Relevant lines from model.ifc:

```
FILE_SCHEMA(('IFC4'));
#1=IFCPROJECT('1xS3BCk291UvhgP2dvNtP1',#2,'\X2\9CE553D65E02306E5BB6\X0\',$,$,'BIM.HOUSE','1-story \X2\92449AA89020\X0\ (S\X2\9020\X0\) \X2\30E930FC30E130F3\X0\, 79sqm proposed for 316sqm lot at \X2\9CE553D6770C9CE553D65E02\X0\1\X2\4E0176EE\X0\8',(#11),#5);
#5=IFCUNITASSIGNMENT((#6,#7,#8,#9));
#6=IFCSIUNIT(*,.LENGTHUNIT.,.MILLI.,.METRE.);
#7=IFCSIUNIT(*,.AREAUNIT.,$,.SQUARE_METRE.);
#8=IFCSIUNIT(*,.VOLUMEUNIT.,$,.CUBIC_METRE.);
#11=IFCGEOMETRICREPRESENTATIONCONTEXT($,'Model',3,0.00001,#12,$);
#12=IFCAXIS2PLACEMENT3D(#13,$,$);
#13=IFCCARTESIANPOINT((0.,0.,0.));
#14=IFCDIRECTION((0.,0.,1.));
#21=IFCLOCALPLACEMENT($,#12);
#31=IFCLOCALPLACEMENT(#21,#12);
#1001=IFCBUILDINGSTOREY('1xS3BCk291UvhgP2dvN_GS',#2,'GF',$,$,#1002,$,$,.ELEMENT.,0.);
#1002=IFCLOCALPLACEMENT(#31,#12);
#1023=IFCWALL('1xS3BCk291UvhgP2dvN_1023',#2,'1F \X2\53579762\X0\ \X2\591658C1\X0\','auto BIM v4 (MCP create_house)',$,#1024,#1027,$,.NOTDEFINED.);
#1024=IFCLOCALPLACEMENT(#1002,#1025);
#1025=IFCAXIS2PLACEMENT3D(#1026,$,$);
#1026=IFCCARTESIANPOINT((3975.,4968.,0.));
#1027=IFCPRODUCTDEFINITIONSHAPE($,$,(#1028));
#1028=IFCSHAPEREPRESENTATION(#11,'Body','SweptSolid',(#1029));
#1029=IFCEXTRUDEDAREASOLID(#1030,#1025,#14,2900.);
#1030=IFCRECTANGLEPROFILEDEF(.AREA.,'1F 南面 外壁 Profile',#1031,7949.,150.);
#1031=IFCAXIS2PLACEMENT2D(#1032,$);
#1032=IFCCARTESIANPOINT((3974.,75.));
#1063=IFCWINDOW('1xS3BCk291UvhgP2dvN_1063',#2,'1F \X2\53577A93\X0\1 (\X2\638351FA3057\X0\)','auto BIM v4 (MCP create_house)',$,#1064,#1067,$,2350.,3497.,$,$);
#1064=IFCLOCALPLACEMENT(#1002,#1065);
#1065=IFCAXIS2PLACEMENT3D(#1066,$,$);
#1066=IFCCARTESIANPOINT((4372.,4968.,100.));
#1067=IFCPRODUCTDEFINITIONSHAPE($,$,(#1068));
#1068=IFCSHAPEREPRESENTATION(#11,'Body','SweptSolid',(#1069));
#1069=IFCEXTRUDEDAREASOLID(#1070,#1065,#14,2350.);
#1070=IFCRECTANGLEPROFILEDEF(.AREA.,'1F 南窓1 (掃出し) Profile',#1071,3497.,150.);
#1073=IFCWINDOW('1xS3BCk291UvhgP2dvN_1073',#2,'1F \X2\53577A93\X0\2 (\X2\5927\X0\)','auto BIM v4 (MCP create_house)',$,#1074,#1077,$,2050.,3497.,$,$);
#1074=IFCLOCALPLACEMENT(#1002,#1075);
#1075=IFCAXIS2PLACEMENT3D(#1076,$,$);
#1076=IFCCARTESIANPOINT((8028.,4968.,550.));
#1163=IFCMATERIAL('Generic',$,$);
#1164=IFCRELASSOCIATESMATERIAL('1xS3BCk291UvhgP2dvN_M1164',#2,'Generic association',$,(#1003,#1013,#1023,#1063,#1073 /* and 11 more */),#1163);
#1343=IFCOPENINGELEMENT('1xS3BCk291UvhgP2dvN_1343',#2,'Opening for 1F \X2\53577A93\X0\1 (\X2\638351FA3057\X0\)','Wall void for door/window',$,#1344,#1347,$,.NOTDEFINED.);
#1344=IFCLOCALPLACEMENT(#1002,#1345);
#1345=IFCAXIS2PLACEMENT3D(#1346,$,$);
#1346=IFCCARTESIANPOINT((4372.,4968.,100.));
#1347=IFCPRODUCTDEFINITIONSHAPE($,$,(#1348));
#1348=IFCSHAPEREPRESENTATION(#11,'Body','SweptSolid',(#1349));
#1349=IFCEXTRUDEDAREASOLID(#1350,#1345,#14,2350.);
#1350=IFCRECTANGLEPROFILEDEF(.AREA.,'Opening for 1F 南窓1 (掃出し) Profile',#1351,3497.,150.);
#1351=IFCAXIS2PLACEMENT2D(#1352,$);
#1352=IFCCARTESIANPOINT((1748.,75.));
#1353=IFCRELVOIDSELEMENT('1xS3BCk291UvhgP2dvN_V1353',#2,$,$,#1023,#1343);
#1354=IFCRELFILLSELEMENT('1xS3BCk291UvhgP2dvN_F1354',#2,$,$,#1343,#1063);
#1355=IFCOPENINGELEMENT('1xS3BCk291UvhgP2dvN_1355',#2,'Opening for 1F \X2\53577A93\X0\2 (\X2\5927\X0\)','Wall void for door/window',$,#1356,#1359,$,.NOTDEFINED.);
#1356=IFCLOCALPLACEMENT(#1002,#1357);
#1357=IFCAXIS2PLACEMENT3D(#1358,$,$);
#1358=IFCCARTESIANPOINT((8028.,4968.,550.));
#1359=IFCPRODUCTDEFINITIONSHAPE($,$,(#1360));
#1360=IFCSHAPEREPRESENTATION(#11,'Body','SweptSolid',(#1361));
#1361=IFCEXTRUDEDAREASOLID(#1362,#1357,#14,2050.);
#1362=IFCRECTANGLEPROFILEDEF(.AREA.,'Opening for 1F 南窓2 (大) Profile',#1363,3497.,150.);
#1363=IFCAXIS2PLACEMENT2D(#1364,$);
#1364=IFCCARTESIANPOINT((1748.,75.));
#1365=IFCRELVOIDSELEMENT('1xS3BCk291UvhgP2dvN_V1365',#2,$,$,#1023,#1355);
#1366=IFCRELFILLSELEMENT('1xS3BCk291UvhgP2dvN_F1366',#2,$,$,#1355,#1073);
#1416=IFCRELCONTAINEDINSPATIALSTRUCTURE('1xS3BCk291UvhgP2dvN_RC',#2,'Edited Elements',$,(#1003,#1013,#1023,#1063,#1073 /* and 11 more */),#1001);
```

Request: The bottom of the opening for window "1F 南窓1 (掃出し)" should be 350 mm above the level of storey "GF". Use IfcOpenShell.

```python
import numpy as np
import ifcopenshell
import ifcopenshell.api.geometry
import ifcopenshell.geom
import ifcopenshell.util.element
import ifcopenshell.util.placement
import ifcopenshell.util.shape
import ifcopenshell.util.unit

model = ifcopenshell.open("model.ifc")
unit_scale = ifcopenshell.util.unit.calculate_unit_scale(model)

window = model.by_guid("1xS3BCk291UvhgP2dvN_1063")
opening = window.FillsVoids[0].RelatingOpeningElement
storey = ifcopenshell.util.element.get_container(window, ifc_class="IfcBuildingStorey")
level = ifcopenshell.util.placement.get_local_placement(storey.ObjectPlacement)[2, 3]

# The opening's origin need not be at the sill, so measure its lowest point.
shape = ifcopenshell.geom.create_shape(ifcopenshell.geom.settings(), opening)
bottom = ifcopenshell.util.shape.get_shape_bottom_elevation(shape, shape.geometry) / unit_scale
dz = level + 0.35 / unit_scale - bottom

shift = np.array([0.0, 0.0, dz])
# The window is not placed relative to its opening, so move both.
for product in (opening, window):
    matrix = ifcopenshell.util.placement.get_local_placement(product.ObjectPlacement)
    matrix[:3, 3] += shift
    ifcopenshell.api.geometry.edit_object_placement(model, product=product, matrix=matrix, is_si=False)

print(f"moved by {dz * unit_scale:+.3f} m")

model.write("model_v2.ifc")
```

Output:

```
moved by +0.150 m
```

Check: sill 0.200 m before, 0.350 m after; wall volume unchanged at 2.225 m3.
